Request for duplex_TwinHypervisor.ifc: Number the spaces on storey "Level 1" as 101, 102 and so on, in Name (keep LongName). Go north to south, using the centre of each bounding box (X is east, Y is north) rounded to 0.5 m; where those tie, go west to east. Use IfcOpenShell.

First a look at what the model holds.

```python
import ifcopenshell
import ifcopenshell.util.element
import ifcopenshell.util.placement

model = ifcopenshell.open("duplex_TwinHypervisor.ifc")
print(model.schema)
storey = next(s for s in model.by_type("IfcBuildingStorey") if s.Name == "Level 1")
spaces = [e for e in ifcopenshell.util.element.get_decomposition(storey) if e.is_a("IfcSpace")]
for e in sorted(spaces, key=lambda e: e.id()):
    origin = ifcopenshell.util.placement.get_local_placement(e.ObjectPlacement)[:3, 3]
    print(e.id(), e.Name, e.LongName, origin.round(2) + 0.0, sep=" | ")
```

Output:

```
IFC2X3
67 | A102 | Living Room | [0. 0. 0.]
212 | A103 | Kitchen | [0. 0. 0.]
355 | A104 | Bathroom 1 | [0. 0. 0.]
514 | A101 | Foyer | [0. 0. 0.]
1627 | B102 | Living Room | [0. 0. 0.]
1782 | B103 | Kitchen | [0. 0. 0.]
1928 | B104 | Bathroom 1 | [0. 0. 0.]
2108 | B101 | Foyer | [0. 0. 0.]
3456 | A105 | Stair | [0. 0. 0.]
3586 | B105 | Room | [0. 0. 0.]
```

```python
import ifcopenshell
import ifcopenshell.geom
import ifcopenshell.util.element
import ifcopenshell.util.shape

model = ifcopenshell.open("duplex_TwinHypervisor.ifc")
settings = ifcopenshell.geom.settings()
settings.set("use-world-coords", True)


def centre(element):
    shape = ifcopenshell.geom.create_shape(settings, element)
    return ifcopenshell.util.shape.get_bbox_centroid(shape.geometry)


storey = next(s for s in model.by_type("IfcBuildingStorey") if s.Name == "Level 1")
spaces = [e for e in ifcopenshell.util.element.get_decomposition(storey) if e.is_a("IfcSpace")]

# Insertion points can sit at a corner or the storey origin, so sort by the geometry (in metres).
centres = {e: centre(e) for e in spaces}
spaces.sort(key=lambda e: (-round(centres[e][1] / 0.5), centres[e][0]))

for i, e in enumerate(spaces, start=1):
    number = f"1{i:02d}"
    e.Name = number
    print(e.id(), number)

model.write("duplex_TwinHypervisor_updated.ifc")
```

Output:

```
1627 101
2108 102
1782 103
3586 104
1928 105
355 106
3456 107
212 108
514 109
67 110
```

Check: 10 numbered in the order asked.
